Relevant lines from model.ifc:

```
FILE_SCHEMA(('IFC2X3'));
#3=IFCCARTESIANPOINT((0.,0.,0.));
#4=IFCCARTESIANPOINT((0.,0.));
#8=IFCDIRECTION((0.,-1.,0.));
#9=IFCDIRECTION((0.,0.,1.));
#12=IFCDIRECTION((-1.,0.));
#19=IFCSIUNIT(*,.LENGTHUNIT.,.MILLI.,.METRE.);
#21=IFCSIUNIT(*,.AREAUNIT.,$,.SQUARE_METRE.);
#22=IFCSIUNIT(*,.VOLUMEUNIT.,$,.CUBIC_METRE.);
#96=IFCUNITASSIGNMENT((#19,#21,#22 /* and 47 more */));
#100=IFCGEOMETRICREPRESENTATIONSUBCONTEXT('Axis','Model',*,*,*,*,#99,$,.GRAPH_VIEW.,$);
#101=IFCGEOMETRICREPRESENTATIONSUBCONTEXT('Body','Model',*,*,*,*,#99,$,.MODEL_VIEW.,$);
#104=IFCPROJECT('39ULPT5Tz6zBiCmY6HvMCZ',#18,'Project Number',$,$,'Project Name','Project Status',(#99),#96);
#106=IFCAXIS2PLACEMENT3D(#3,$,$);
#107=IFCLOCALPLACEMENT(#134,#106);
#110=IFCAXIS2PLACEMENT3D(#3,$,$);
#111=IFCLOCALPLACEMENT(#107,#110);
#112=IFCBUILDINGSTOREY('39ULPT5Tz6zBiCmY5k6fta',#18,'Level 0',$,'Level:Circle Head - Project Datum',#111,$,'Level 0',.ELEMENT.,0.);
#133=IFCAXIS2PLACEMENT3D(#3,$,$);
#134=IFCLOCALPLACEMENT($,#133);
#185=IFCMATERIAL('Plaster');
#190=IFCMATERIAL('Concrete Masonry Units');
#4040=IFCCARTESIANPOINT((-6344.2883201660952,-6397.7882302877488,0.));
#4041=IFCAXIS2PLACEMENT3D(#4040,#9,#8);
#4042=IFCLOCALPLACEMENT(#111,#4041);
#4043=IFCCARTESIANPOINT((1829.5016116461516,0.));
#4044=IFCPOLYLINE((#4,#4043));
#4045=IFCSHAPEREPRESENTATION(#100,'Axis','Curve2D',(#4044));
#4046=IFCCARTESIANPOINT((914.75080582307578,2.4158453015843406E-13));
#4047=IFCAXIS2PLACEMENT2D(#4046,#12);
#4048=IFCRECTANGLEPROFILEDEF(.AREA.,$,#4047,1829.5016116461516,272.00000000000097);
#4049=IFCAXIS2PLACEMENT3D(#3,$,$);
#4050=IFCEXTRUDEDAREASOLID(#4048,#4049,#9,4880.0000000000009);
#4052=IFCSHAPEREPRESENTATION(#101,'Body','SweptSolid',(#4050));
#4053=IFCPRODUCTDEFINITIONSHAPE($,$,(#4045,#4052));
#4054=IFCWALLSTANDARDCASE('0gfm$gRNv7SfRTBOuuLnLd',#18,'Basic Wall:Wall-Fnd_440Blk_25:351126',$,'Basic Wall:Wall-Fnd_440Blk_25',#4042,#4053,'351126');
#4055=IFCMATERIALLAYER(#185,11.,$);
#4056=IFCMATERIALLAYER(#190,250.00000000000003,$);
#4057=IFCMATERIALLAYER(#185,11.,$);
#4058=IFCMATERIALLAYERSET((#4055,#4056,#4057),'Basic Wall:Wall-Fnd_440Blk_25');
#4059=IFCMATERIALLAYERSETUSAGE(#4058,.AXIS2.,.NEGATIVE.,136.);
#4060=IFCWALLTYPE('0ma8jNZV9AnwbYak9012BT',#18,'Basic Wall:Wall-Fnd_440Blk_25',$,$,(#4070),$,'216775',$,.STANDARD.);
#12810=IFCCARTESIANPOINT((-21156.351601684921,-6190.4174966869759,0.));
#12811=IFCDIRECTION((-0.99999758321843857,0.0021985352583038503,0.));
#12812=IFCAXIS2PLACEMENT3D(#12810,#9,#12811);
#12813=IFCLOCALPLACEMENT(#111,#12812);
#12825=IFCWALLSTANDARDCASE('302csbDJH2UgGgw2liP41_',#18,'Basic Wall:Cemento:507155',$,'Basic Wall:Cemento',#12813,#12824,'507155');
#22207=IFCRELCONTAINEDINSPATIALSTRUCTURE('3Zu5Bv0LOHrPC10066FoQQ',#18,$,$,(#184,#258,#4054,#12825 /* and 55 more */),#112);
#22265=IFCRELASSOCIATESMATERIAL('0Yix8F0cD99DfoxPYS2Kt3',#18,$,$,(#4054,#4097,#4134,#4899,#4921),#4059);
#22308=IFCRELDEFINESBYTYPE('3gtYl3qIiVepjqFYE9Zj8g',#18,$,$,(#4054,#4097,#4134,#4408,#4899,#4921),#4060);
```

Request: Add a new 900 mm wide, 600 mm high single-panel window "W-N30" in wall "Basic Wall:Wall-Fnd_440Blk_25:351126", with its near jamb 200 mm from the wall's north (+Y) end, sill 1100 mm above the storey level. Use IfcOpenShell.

```python
import numpy as np
import ifcopenshell
import ifcopenshell.api.feature
import ifcopenshell.api.geometry
import ifcopenshell.api.root
import ifcopenshell.api.spatial
import ifcopenshell.api.type
import ifcopenshell.geom
import ifcopenshell.util.element
import ifcopenshell.util.placement
import ifcopenshell.util.representation
import ifcopenshell.util.shape
import ifcopenshell.util.unit

model = ifcopenshell.open("model.ifc")
unit_scale = ifcopenshell.util.unit.calculate_unit_scale(model)
settings = ifcopenshell.geom.settings()


def volume(element):
    """Net volume in cubic metres, openings subtracted."""
    shape = ifcopenshell.geom.create_shape(settings, element)
    return ifcopenshell.util.shape.get_volume(shape.geometry)


wall = model.by_id(4054)
storey = ifcopenshell.util.element.get_container(wall, ifc_class="IfcBuildingStorey")
context = ifcopenshell.util.representation.get_context(model, "Model", "Body", "MODEL_VIEW")
before = volume(wall)

width, height, from_end, sill = 0.9, 0.6, 0.2, 1.1  # metres

# The wall runs along its own X axis, and the end named is its -X end.
wall_shape = ifcopenshell.geom.create_shape(settings, wall)
x, y, z = ifcopenshell.util.shape.get_vertices(wall_shape.geometry).T
start = x.min() + from_end
face, thickness = float(y.min()), float(y.max() - y.min())
wall_matrix = ifcopenshell.util.placement.get_local_placement(wall.ObjectPlacement)
level = ifcopenshell.util.placement.get_local_placement(storey.ObjectPlacement)[2, 3]


def in_wall(x, y):
    """Placement at x, y metres in the wall's axes, at sill height."""
    matrix = wall_matrix.copy()
    matrix[:, 3] = wall_matrix @ np.array([x / unit_scale, y / unit_scale, 0.0, 1.0])
    matrix[2, 3] = level + sill / unit_scale
    return matrix


# Opening: a box that overshoots both wall faces by 50 mm.
opening = ifcopenshell.api.root.create_entity(model, ifc_class="IfcOpeningElement")
box = ifcopenshell.api.geometry.add_wall_representation(
    model, context=context, length=width, height=height, thickness=thickness + 0.1
)
ifcopenshell.api.geometry.assign_representation(model, product=opening, representation=box)
ifcopenshell.api.geometry.edit_object_placement(model, product=opening, matrix=in_wall(start, face - 0.05), is_si=False)
ifcopenshell.api.feature.add_feature(model, feature=opening, element=wall)

window = ifcopenshell.api.root.create_entity(model, ifc_class="IfcWindow", name="W-N30")
window.OverallWidth, window.OverallHeight = width / unit_scale, height / unit_scale
body = ifcopenshell.api.geometry.add_window_representation(
    model,
    context=context,
    overall_width=window.OverallWidth,
    overall_height=window.OverallHeight,
    partition_type="SINGLE_PANEL",
)
ifcopenshell.api.geometry.assign_representation(model, product=window, representation=body)
ifcopenshell.api.spatial.assign_container(model, products=[window], relating_structure=storey)
fills = ifcopenshell.api.feature.add_filling(model, opening=opening, element=window)
fills.OwnerHistory = window.OwnerHistory  # required in IFC2X3

# IFC2X3 keeps the operation on the window style.
style = ifcopenshell.api.root.create_entity(model, ifc_class="IfcWindowStyle", name="W-N30")
style.OperationType, style.ConstructionType = "SINGLE_PANEL", "NOTDEFINED"
style.ParameterTakesPrecedence = style.Sizeable = False
ifcopenshell.api.type.assign_type(model, related_objects=[window], relating_type=style)

# Centre the window in the wall's thickness.
ifcopenshell.api.geometry.edit_object_placement(model, product=window, matrix=in_wall(start, face), is_si=False)
window_shape = ifcopenshell.geom.create_shape(settings, window)
depth = ifcopenshell.util.shape.get_vertices(window_shape.geometry)[:, 1]
offset = face + thickness / 2 - (depth.min() + depth.max()) / 2
ifcopenshell.api.geometry.edit_object_placement(model, product=window, matrix=in_wall(start, offset), is_si=False)

after = volume(wall)

print(f"wall volume {before:.3f} -> {after:.3f} m3")

model.write("model-out.ifc")
```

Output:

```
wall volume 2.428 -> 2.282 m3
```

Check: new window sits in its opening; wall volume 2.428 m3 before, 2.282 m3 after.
